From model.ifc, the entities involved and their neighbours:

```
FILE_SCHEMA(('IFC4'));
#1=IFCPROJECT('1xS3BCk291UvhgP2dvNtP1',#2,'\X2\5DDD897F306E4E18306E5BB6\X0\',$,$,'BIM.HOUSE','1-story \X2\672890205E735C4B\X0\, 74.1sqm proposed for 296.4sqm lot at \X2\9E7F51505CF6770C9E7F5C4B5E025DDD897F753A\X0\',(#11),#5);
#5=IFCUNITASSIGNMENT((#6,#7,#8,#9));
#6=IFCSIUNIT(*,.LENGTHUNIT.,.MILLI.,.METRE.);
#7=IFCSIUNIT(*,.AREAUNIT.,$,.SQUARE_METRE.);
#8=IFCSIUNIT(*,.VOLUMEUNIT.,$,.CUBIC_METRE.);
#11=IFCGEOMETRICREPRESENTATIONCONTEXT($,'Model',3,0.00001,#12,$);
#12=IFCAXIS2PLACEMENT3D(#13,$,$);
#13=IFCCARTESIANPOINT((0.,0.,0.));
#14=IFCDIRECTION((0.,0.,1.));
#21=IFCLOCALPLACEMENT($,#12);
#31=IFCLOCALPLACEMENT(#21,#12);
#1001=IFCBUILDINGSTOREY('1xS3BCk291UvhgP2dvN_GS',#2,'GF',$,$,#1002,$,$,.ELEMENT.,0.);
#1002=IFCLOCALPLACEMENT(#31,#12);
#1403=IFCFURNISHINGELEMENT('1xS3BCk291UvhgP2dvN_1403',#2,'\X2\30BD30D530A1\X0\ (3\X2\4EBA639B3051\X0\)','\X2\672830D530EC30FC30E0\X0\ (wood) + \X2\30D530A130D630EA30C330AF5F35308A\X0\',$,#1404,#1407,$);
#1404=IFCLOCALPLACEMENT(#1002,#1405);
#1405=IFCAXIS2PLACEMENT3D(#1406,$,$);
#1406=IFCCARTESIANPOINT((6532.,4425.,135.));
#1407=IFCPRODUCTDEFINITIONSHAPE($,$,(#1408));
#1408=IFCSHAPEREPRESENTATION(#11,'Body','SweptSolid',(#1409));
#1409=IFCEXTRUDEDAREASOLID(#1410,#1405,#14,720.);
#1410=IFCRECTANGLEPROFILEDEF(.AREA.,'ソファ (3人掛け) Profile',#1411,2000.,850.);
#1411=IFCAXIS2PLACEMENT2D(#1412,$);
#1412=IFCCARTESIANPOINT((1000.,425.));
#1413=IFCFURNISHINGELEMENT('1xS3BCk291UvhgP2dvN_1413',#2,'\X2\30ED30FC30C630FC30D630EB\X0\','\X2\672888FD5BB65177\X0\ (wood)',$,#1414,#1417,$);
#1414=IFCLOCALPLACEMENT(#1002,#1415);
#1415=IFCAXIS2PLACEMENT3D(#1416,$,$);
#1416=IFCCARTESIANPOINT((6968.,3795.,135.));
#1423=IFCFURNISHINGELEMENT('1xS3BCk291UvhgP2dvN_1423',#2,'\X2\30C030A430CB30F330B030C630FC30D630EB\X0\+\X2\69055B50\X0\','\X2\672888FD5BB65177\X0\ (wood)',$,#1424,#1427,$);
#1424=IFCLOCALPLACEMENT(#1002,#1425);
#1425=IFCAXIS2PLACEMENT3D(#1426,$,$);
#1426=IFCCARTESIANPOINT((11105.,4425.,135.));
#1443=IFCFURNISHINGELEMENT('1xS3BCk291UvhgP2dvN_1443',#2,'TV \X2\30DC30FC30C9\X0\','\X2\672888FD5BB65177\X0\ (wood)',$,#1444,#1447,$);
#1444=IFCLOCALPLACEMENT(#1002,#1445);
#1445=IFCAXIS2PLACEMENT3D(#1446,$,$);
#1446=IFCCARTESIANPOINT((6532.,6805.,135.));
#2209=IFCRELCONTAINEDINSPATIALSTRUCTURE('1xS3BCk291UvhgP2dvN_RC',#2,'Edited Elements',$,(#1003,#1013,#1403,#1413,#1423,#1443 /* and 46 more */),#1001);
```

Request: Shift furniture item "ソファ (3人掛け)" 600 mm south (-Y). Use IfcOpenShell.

```python
import ifcopenshell
import ifcopenshell.api.geometry
import ifcopenshell.util.placement
import ifcopenshell.util.unit

model = ifcopenshell.open("model.ifc")
unit_scale = ifcopenshell.util.unit.calculate_unit_scale(model)

item = model.by_id(1403)
matrix = ifcopenshell.util.placement.get_local_placement(item.ObjectPlacement)
matrix[1, 3] -= 0.6 / unit_scale
ifcopenshell.api.geometry.edit_object_placement(model, product=item, matrix=matrix, is_si=False)

print(ifcopenshell.util.placement.get_local_placement(item.ObjectPlacement).round(3) + 0.0)

model.write("model_rev.ifc")
```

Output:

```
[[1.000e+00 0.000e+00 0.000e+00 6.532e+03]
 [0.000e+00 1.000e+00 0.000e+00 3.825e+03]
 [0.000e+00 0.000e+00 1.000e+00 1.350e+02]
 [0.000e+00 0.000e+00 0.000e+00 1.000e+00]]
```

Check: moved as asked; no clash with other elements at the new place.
